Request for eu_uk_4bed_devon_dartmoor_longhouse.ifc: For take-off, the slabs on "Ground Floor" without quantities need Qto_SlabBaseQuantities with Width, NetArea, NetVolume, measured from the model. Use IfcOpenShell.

First a look at what the model holds.

```python
import ifcopenshell
import ifcopenshell.util.element
import ifcopenshell.util.unit

model = ifcopenshell.open("eu_uk_4bed_devon_dartmoor_longhouse.ifc")
print(model.schema)
for unit_type in ("LENGTHUNIT", "AREAUNIT", "VOLUMEUNIT"):
    print(unit_type, ifcopenshell.util.unit.calculate_unit_scale(model, unit_type))
storey = next(s for s in model.by_type("IfcBuildingStorey") if s.Name == "Ground Floor")
slabs = [e for e in ifcopenshell.util.element.get_decomposition(storey) if e.is_a("IfcSlab")]
for e in sorted(slabs, key=lambda e: e.id()):
    print(e.id(), e.is_a(), e.Name, list(ifcopenshell.util.element.get_psets(e, qtos_only=True)), sep=" | ")
```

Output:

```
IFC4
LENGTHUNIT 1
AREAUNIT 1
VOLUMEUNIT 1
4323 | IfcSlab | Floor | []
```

```python
import ifcopenshell
import ifcopenshell.api.pset
import ifcopenshell.geom
import ifcopenshell.util.element
import ifcopenshell.util.shape
import ifcopenshell.util.unit

model = ifcopenshell.open("eu_uk_4bed_devon_dartmoor_longhouse.ifc")
unit_scale = ifcopenshell.util.unit.calculate_unit_scale(model)
area_scale = ifcopenshell.util.unit.calculate_unit_scale(model, "AREAUNIT")
volume_scale = ifcopenshell.util.unit.calculate_unit_scale(model, "VOLUMEUNIT")
settings = ifcopenshell.geom.settings()

storey = next(s for s in model.by_type("IfcBuildingStorey") if s.Name == "Ground Floor")
slabs = [e for e in ifcopenshell.util.element.get_decomposition(storey) if e.is_a("IfcSlab")]

for e in sorted(slabs, key=lambda e: e.id()):
    if ifcopenshell.util.element.get_psets(e, qtos_only=True, should_inherit=False):
        continue
    # Geometry comes back in metres, in the element's own axes.
    shape = ifcopenshell.geom.create_shape(settings, e)
    values = {
        "Width": ifcopenshell.util.shape.get_z(shape.geometry) / unit_scale,
        "NetArea": ifcopenshell.util.shape.get_footprint_area(shape.geometry) / area_scale,
        "NetVolume": ifcopenshell.util.shape.get_volume(shape.geometry) / volume_scale,
    }
    qto = ifcopenshell.api.pset.add_qto(model, product=e, name="Qto_SlabBaseQuantities")
    ifcopenshell.api.pset.edit_qto(model, qto=qto, properties=values)
    print(e.id(), {k: round(v, 3) for k, v in values.items()})

model.write("eu_uk_4bed_devon_dartmoor_longhouse_updated.ifc")
```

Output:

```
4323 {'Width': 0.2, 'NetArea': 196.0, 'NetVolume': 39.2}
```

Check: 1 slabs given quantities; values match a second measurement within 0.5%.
